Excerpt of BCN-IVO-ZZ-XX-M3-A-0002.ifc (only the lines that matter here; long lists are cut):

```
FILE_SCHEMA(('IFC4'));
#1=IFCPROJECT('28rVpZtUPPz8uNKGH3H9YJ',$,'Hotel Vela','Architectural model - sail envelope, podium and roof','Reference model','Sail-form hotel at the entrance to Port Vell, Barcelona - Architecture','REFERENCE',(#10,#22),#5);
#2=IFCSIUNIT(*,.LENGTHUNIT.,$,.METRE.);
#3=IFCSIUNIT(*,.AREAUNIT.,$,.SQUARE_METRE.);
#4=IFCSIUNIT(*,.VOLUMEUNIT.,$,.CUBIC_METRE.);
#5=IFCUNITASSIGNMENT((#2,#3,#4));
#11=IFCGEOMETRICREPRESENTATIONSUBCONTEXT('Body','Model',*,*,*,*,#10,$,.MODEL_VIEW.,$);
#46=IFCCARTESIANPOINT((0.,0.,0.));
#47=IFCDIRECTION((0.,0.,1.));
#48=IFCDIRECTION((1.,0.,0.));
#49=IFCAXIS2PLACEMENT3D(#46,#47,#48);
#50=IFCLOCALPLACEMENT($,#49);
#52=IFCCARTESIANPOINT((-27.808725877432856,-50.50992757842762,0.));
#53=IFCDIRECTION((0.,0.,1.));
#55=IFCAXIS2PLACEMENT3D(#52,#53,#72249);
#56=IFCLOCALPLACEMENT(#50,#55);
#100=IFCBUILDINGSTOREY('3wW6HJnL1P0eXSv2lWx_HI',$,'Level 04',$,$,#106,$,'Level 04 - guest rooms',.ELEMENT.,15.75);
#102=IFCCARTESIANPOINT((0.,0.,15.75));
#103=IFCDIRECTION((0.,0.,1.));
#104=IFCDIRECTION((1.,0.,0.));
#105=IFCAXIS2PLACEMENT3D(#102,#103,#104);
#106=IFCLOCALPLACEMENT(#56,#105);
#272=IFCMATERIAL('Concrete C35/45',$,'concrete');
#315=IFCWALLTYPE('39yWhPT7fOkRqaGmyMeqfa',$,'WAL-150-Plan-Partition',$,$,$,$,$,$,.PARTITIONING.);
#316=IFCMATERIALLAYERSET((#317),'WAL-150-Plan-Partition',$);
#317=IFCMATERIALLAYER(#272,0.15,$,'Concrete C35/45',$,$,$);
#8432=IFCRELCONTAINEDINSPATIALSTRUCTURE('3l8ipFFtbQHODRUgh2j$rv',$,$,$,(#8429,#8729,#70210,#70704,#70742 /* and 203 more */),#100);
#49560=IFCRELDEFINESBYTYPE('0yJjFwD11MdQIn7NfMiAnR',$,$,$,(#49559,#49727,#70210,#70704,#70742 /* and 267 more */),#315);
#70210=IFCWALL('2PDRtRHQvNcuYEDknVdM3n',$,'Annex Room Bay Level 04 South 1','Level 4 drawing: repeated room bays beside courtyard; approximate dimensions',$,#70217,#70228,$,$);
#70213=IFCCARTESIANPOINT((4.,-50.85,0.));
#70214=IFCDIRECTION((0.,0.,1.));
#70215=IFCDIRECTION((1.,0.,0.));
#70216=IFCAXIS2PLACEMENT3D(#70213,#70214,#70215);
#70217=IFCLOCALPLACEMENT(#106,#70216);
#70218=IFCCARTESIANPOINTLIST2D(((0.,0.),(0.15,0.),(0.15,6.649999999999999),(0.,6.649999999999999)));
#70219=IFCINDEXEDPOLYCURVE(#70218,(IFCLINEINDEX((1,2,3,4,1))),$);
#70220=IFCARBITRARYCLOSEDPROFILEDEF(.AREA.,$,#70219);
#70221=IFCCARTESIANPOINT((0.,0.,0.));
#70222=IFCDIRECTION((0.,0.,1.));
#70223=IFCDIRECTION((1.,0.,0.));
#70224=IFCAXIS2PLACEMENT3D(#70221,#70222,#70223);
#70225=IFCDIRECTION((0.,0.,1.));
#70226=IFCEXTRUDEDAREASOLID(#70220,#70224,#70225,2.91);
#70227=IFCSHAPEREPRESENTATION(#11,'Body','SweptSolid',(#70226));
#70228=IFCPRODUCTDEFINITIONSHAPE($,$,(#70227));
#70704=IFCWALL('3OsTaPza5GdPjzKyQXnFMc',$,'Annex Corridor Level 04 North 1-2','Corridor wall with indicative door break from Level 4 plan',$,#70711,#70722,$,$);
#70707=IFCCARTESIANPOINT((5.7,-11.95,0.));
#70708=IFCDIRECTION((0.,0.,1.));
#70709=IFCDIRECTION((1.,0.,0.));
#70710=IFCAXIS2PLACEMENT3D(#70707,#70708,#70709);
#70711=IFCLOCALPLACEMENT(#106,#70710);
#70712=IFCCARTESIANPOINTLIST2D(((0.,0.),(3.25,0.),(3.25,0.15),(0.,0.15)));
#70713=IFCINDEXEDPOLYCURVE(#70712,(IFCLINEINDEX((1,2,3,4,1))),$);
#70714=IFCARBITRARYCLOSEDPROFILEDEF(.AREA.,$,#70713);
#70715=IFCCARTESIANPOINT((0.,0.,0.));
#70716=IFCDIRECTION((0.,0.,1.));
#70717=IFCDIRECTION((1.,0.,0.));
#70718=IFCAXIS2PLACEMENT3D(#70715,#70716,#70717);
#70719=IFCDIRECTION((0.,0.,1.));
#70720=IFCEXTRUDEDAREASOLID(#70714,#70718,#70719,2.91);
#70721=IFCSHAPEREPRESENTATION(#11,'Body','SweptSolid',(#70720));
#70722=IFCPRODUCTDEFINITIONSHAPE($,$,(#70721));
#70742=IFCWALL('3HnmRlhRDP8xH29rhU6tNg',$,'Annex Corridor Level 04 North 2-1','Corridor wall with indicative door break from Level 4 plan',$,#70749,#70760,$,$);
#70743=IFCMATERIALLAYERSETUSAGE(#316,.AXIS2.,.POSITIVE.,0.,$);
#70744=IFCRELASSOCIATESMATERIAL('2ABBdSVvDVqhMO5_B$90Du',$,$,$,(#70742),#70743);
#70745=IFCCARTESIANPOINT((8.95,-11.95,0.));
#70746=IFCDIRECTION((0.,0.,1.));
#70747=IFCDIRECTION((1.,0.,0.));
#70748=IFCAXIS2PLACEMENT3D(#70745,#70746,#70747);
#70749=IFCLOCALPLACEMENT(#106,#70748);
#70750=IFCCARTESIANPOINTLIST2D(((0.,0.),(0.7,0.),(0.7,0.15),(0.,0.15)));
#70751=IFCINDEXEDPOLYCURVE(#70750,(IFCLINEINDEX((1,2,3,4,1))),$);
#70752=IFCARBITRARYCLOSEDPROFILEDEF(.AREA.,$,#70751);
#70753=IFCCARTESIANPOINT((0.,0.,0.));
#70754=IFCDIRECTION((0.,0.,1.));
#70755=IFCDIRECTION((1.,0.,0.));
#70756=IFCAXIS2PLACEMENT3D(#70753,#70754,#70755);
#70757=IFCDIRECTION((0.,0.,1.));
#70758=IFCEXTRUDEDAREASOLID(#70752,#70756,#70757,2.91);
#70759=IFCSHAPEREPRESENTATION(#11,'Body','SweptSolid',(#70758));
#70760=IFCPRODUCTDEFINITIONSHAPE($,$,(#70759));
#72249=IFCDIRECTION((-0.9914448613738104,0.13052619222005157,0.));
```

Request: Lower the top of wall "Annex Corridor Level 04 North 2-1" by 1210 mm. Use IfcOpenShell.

```python
import ifcopenshell
import ifcopenshell.geom
import ifcopenshell.util.representation
import ifcopenshell.util.shape

model = ifcopenshell.open("BCN-IVO-ZZ-XX-M3-A-0002.ifc")
settings = ifcopenshell.geom.settings()


def volume(element):
    """Net volume in cubic metres, openings subtracted."""
    shape = ifcopenshell.geom.create_shape(settings, element)
    return ifcopenshell.util.shape.get_volume(shape.geometry)


wall = model.by_guid("3HnmRlhRDP8xH29rhU6tNg")
before = volume(wall)

body = ifcopenshell.util.representation.get_representation(wall, "Model", "Body")
solid = body.Items[0]
old_height = solid.Depth
solid.Depth -= 1.21
after = volume(wall)

print(f"height {old_height:g} -> {solid.Depth:g}, volume {before:.3f} -> {after:.3f} m3")

model.write("BCN-IVO-ZZ-XX-M3-A-0002_rev.ifc")
```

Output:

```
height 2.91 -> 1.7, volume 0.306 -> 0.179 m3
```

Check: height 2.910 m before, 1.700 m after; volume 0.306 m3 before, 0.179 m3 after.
